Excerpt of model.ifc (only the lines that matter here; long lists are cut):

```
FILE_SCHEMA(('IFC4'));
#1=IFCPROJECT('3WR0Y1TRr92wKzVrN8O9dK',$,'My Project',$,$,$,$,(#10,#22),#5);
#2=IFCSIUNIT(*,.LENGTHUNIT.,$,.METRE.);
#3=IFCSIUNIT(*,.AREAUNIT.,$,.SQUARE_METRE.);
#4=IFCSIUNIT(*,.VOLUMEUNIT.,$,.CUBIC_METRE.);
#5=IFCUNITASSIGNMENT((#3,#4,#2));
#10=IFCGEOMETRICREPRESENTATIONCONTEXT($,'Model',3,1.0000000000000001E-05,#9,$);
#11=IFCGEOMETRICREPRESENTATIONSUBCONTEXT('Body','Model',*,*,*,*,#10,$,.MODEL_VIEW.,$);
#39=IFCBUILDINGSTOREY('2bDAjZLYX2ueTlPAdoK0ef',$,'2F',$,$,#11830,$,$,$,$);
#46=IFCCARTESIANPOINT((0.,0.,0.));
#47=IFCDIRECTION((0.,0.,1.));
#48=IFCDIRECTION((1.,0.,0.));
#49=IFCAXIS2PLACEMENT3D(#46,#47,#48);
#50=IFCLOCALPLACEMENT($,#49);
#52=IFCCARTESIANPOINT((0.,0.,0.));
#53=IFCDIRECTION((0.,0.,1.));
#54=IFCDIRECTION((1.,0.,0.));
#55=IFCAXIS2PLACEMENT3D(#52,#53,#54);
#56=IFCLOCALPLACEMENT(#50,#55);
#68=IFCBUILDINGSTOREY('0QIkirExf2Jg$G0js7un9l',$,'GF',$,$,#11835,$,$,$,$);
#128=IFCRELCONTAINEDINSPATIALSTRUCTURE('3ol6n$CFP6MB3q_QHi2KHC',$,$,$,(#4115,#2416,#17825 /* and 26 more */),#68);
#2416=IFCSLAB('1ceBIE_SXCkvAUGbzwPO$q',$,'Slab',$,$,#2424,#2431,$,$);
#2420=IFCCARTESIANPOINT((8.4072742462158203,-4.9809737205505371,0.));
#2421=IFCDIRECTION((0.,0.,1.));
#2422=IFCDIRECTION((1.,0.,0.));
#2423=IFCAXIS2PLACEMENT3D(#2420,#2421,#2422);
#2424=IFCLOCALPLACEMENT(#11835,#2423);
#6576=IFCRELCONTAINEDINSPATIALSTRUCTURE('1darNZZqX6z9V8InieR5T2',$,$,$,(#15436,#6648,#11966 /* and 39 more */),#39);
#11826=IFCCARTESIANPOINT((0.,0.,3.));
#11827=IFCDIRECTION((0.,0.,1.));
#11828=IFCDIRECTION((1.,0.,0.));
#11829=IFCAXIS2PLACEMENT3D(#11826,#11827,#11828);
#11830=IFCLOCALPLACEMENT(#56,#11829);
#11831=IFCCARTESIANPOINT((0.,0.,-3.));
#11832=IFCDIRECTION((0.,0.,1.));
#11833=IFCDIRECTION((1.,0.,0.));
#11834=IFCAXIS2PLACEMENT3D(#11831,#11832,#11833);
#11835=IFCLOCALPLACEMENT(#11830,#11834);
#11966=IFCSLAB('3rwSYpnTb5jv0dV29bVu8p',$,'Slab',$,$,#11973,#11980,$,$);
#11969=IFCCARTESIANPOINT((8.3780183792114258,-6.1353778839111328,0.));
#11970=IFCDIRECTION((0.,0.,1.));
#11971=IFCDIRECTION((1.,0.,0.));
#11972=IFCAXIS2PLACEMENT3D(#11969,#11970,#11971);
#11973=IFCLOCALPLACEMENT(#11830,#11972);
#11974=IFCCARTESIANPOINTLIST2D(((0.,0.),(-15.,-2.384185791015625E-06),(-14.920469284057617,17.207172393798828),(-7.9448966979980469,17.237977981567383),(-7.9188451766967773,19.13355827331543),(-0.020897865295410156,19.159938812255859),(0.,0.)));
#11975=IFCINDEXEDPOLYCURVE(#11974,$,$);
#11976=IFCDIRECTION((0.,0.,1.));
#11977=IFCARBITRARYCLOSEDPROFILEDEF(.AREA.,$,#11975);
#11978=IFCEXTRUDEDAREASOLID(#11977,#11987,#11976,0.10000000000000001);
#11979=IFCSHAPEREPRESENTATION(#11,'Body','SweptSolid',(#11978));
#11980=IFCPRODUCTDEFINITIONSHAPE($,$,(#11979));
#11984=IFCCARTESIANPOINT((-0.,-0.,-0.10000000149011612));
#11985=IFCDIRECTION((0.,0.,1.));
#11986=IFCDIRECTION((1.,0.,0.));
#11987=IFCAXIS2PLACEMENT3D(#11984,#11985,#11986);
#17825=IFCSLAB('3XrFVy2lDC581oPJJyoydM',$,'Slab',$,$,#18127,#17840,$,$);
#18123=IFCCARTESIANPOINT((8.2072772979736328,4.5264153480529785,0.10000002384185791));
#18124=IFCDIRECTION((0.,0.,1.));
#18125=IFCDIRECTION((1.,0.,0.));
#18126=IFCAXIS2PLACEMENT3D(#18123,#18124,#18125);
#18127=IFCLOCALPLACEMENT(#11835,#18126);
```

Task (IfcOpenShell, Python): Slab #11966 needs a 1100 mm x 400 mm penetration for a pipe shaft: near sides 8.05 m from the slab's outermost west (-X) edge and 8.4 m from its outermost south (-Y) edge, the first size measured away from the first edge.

```python
import numpy as np
import ifcopenshell
import ifcopenshell.api.feature
import ifcopenshell.api.geometry
import ifcopenshell.api.root
import ifcopenshell.geom
import ifcopenshell.util.placement
import ifcopenshell.util.representation
import ifcopenshell.util.shape
import ifcopenshell.util.unit

model = ifcopenshell.open("model.ifc")
unit_scale = ifcopenshell.util.unit.calculate_unit_scale(model)
settings = ifcopenshell.geom.settings()


def volume(element):
    """Net volume in cubic metres, openings subtracted."""
    shape = ifcopenshell.geom.create_shape(settings, element)
    return ifcopenshell.util.shape.get_volume(shape.geometry)


slab = model.by_guid("3rwSYpnTb5jv0dV29bVu8p")
before = volume(slab)

# Extent in the slab's own axes, in metres. The edges named are its -X and -Y sides.
slab_shape = ifcopenshell.geom.create_shape(settings, slab)
vertices = ifcopenshell.util.shape.get_vertices(slab_shape.geometry)
x_min, y_min, bottom = vertices.min(axis=0)
top = vertices[:, 2].max()

opening = ifcopenshell.api.root.create_entity(model, ifc_class="IfcOpeningElement", name="Pipe shaft opening", predefined_type="OPENING")
context = ifcopenshell.util.representation.get_context(model, "Model", "Body", "MODEL_VIEW")
width, depth = 1.1, 0.4
outline = [(0.0, 0.0), (width, 0.0), (width, depth), (0.0, depth), (0.0, 0.0)]
# Overshoot both faces by 50 mm so the cut is clean.
shape = ifcopenshell.api.geometry.add_slab_representation(
    model, context=context, depth=top - bottom + 0.1, polyline=outline
)
ifcopenshell.api.geometry.assign_representation(model, product=opening, representation=shape)

matrix = ifcopenshell.util.placement.get_local_placement(slab.ObjectPlacement)
matrix[:, 3] = matrix @ np.append(np.array([x_min + 8.05, y_min + 8.4, bottom - 0.05]) / unit_scale, 1.0)
ifcopenshell.api.geometry.edit_object_placement(model, product=opening, matrix=matrix, is_si=False)
ifcopenshell.api.feature.add_feature(model, feature=opening, element=slab)

after = volume(slab)

print(f"slab volume {before:.3f} -> {after:.3f} m3")

model.write("model_rev.ifc")
```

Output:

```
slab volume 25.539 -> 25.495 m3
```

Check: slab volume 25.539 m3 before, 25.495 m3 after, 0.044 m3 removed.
